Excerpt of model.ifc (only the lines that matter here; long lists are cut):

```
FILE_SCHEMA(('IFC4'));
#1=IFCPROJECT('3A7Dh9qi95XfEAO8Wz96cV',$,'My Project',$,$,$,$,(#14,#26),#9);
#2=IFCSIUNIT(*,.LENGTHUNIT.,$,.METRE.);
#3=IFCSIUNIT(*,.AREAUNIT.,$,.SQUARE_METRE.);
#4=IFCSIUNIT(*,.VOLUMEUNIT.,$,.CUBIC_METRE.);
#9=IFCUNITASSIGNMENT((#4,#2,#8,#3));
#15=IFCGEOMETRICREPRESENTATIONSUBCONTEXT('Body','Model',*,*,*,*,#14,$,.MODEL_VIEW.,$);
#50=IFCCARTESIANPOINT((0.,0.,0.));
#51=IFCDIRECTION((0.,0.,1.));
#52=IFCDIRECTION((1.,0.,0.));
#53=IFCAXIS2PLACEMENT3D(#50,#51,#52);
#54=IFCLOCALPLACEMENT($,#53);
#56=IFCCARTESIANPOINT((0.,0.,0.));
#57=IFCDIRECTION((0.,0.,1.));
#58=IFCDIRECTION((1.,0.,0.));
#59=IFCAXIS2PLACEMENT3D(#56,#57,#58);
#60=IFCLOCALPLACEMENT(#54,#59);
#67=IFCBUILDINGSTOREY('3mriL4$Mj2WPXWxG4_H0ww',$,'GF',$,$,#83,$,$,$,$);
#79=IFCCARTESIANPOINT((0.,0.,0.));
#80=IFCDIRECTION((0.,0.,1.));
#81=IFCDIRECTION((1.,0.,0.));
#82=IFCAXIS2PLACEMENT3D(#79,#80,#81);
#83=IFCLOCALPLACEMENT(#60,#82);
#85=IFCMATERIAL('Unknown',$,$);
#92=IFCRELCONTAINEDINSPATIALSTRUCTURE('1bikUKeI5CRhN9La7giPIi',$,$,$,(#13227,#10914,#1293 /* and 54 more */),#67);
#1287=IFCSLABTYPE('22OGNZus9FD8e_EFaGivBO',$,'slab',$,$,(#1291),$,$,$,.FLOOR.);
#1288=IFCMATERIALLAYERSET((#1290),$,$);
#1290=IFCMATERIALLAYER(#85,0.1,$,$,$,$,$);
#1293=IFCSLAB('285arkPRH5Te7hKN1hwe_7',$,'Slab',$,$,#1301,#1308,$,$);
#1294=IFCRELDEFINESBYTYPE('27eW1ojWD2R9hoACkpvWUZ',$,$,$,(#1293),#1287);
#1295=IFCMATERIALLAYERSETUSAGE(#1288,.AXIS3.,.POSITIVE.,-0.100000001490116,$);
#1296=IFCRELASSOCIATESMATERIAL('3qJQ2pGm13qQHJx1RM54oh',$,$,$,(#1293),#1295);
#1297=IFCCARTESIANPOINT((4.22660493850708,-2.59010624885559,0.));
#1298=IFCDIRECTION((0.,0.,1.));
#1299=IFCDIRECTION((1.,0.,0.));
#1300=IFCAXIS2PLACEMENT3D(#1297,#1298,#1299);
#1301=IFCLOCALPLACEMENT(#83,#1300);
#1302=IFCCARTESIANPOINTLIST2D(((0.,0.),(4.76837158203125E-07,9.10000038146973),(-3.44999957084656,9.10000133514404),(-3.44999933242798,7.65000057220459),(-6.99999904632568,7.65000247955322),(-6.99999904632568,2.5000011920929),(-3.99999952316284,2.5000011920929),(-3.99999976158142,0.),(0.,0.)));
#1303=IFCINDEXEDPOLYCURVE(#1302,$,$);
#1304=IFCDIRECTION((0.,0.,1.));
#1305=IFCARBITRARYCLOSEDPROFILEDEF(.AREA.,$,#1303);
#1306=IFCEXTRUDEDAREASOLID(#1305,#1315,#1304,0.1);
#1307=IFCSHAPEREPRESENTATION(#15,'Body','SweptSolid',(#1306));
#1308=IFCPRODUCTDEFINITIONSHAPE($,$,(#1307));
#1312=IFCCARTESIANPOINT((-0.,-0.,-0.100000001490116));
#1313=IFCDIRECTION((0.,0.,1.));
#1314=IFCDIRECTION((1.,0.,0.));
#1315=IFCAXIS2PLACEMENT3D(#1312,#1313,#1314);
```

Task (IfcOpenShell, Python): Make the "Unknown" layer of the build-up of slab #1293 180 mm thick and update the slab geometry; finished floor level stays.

```python
import ifcopenshell
import ifcopenshell.util.element
import ifcopenshell.util.representation

model = ifcopenshell.open("model.ifc")

layer_set = model.by_id(1288)
layer = next(l for l in layer_set.MaterialLayers if l.Material and l.Material.Name == "Unknown")
change = 0.18 - layer.LayerThickness
layer.LayerThickness += change

# Geometry does not follow the layer set by itself.
slabs = [e for e in ifcopenshell.util.element.get_elements_by_material(model, layer_set) if e.is_a("IfcSlab")]
for slab in sorted(slabs, key=lambda e: e.id()):
    body = ifcopenshell.util.representation.get_representation(slab, "Model", "Body")
    solid = body.Items[0]
    old_depth = solid.Depth
    solid.Depth += change
    # Extruded upwards: lower the start of the extrusion so the top stays.
    x, y, z = solid.Position.Location.Coordinates
    solid.Position.Location = model.createIfcCartesianPoint((x, y, z - change))
    print(slab.id(), f"{old_depth:g} -> {solid.Depth:g}")

# The layers are counted up from the underside, which has moved.
for usage in {ifcopenshell.util.element.get_material(slab) for slab in slabs}:
    usage.OffsetFromReferenceLine -= change

model.write("model_edited.ifc")
```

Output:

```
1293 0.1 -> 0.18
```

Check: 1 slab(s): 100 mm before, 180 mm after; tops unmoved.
